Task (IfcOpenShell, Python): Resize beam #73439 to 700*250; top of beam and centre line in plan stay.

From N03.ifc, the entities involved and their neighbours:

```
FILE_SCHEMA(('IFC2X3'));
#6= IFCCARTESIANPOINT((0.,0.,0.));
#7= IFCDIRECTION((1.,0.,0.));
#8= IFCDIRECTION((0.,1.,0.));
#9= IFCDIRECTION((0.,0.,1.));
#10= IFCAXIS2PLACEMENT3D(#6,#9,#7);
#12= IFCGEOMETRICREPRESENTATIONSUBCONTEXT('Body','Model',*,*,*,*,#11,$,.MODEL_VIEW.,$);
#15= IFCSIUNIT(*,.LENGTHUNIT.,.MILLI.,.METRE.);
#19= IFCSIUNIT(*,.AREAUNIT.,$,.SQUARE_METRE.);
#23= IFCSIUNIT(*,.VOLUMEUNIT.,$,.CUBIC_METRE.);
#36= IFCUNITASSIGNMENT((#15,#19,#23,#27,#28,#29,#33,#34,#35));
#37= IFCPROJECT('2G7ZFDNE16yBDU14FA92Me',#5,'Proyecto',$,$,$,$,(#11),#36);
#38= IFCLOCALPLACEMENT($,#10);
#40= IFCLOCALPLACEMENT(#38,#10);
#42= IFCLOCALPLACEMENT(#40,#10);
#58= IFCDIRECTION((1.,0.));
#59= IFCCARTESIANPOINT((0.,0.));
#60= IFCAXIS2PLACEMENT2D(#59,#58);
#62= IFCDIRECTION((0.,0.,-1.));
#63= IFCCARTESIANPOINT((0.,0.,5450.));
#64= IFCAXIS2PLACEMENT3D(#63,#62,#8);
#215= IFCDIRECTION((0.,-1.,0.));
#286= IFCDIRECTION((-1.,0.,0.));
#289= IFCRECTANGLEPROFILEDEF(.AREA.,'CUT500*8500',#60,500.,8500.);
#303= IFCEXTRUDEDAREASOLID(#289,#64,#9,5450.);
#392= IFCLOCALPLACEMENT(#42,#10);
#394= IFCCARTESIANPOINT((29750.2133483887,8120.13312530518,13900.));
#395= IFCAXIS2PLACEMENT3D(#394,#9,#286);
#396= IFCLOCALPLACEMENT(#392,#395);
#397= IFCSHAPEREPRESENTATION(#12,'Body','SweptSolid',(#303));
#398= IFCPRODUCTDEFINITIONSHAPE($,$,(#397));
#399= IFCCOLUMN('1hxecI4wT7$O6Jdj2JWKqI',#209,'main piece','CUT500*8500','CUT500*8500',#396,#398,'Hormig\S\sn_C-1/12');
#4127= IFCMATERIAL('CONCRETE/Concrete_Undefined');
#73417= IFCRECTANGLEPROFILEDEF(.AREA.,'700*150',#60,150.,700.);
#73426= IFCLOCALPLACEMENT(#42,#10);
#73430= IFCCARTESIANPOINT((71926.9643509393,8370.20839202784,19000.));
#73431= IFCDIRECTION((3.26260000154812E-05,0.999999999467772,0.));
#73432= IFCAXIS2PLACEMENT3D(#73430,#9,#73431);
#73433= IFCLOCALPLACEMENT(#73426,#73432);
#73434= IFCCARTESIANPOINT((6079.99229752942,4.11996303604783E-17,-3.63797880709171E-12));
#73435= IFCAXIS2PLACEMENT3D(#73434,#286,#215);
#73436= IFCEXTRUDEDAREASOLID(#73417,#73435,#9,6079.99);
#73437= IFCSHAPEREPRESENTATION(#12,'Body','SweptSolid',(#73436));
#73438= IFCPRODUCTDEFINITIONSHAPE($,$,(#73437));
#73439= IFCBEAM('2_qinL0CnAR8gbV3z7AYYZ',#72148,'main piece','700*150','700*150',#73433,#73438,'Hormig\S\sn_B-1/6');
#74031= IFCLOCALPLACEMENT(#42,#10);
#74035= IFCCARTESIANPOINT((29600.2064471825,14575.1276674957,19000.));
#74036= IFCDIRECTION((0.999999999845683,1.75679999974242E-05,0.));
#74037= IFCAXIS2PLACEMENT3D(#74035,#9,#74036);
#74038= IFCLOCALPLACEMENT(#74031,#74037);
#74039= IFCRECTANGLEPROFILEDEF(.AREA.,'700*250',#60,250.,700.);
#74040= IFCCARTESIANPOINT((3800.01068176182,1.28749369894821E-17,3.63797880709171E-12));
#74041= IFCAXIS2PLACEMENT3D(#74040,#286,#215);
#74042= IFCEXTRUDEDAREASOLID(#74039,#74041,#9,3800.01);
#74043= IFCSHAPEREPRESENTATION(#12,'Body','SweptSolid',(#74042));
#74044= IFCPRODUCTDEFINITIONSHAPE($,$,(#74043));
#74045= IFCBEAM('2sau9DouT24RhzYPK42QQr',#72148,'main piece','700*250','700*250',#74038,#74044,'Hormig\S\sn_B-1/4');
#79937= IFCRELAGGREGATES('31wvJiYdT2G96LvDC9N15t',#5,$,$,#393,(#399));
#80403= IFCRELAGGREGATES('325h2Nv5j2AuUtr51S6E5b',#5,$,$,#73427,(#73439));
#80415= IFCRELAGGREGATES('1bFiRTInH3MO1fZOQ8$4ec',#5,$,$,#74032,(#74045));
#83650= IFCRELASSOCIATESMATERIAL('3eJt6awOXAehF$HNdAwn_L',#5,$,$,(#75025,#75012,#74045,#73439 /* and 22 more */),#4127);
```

```python
import ifcopenshell
import ifcopenshell.util.element
import ifcopenshell.util.representation

model = ifcopenshell.open("N03.ifc")

member = model.by_id(73439)
source = next(p for p in model.by_type("IfcRectangleProfileDef") if p.ProfileName == "700*250")

body = ifcopenshell.util.representation.get_representation(member, "Model", "Body")
solid = body.Items[0]
old_profile = solid.SweptArea

# Copy the section's sizes but keep this member's own profile position.
profile = ifcopenshell.util.element.copy(model, source)
# Profiles are centred, so shift by half the change in depth to hold the top.
shift = (old_profile.YDim - profile.YDim) / 2
x, y = old_profile.Position.Location.Coordinates
up = (0.0, 1.0)  # upwards, in the solid's own plane
location = model.createIfcCartesianPoint((x + up[0] * shift, y + up[1] * shift))
profile.Position = model.createIfcAxis2Placement2D(location, old_profile.Position.RefDirection)
solid.SweptArea = profile
if not model.get_total_inverses(old_profile):
    ifcopenshell.util.element.remove_deep2(model, old_profile)
member.Description = member.Description.replace("700*150", "700*250")
member.ObjectType = member.ObjectType.replace("700*150", "700*250")

print(solid.SweptArea)

model.write("N03-out.ifc")
```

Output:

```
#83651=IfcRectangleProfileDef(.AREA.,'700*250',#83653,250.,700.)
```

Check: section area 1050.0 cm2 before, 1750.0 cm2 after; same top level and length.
